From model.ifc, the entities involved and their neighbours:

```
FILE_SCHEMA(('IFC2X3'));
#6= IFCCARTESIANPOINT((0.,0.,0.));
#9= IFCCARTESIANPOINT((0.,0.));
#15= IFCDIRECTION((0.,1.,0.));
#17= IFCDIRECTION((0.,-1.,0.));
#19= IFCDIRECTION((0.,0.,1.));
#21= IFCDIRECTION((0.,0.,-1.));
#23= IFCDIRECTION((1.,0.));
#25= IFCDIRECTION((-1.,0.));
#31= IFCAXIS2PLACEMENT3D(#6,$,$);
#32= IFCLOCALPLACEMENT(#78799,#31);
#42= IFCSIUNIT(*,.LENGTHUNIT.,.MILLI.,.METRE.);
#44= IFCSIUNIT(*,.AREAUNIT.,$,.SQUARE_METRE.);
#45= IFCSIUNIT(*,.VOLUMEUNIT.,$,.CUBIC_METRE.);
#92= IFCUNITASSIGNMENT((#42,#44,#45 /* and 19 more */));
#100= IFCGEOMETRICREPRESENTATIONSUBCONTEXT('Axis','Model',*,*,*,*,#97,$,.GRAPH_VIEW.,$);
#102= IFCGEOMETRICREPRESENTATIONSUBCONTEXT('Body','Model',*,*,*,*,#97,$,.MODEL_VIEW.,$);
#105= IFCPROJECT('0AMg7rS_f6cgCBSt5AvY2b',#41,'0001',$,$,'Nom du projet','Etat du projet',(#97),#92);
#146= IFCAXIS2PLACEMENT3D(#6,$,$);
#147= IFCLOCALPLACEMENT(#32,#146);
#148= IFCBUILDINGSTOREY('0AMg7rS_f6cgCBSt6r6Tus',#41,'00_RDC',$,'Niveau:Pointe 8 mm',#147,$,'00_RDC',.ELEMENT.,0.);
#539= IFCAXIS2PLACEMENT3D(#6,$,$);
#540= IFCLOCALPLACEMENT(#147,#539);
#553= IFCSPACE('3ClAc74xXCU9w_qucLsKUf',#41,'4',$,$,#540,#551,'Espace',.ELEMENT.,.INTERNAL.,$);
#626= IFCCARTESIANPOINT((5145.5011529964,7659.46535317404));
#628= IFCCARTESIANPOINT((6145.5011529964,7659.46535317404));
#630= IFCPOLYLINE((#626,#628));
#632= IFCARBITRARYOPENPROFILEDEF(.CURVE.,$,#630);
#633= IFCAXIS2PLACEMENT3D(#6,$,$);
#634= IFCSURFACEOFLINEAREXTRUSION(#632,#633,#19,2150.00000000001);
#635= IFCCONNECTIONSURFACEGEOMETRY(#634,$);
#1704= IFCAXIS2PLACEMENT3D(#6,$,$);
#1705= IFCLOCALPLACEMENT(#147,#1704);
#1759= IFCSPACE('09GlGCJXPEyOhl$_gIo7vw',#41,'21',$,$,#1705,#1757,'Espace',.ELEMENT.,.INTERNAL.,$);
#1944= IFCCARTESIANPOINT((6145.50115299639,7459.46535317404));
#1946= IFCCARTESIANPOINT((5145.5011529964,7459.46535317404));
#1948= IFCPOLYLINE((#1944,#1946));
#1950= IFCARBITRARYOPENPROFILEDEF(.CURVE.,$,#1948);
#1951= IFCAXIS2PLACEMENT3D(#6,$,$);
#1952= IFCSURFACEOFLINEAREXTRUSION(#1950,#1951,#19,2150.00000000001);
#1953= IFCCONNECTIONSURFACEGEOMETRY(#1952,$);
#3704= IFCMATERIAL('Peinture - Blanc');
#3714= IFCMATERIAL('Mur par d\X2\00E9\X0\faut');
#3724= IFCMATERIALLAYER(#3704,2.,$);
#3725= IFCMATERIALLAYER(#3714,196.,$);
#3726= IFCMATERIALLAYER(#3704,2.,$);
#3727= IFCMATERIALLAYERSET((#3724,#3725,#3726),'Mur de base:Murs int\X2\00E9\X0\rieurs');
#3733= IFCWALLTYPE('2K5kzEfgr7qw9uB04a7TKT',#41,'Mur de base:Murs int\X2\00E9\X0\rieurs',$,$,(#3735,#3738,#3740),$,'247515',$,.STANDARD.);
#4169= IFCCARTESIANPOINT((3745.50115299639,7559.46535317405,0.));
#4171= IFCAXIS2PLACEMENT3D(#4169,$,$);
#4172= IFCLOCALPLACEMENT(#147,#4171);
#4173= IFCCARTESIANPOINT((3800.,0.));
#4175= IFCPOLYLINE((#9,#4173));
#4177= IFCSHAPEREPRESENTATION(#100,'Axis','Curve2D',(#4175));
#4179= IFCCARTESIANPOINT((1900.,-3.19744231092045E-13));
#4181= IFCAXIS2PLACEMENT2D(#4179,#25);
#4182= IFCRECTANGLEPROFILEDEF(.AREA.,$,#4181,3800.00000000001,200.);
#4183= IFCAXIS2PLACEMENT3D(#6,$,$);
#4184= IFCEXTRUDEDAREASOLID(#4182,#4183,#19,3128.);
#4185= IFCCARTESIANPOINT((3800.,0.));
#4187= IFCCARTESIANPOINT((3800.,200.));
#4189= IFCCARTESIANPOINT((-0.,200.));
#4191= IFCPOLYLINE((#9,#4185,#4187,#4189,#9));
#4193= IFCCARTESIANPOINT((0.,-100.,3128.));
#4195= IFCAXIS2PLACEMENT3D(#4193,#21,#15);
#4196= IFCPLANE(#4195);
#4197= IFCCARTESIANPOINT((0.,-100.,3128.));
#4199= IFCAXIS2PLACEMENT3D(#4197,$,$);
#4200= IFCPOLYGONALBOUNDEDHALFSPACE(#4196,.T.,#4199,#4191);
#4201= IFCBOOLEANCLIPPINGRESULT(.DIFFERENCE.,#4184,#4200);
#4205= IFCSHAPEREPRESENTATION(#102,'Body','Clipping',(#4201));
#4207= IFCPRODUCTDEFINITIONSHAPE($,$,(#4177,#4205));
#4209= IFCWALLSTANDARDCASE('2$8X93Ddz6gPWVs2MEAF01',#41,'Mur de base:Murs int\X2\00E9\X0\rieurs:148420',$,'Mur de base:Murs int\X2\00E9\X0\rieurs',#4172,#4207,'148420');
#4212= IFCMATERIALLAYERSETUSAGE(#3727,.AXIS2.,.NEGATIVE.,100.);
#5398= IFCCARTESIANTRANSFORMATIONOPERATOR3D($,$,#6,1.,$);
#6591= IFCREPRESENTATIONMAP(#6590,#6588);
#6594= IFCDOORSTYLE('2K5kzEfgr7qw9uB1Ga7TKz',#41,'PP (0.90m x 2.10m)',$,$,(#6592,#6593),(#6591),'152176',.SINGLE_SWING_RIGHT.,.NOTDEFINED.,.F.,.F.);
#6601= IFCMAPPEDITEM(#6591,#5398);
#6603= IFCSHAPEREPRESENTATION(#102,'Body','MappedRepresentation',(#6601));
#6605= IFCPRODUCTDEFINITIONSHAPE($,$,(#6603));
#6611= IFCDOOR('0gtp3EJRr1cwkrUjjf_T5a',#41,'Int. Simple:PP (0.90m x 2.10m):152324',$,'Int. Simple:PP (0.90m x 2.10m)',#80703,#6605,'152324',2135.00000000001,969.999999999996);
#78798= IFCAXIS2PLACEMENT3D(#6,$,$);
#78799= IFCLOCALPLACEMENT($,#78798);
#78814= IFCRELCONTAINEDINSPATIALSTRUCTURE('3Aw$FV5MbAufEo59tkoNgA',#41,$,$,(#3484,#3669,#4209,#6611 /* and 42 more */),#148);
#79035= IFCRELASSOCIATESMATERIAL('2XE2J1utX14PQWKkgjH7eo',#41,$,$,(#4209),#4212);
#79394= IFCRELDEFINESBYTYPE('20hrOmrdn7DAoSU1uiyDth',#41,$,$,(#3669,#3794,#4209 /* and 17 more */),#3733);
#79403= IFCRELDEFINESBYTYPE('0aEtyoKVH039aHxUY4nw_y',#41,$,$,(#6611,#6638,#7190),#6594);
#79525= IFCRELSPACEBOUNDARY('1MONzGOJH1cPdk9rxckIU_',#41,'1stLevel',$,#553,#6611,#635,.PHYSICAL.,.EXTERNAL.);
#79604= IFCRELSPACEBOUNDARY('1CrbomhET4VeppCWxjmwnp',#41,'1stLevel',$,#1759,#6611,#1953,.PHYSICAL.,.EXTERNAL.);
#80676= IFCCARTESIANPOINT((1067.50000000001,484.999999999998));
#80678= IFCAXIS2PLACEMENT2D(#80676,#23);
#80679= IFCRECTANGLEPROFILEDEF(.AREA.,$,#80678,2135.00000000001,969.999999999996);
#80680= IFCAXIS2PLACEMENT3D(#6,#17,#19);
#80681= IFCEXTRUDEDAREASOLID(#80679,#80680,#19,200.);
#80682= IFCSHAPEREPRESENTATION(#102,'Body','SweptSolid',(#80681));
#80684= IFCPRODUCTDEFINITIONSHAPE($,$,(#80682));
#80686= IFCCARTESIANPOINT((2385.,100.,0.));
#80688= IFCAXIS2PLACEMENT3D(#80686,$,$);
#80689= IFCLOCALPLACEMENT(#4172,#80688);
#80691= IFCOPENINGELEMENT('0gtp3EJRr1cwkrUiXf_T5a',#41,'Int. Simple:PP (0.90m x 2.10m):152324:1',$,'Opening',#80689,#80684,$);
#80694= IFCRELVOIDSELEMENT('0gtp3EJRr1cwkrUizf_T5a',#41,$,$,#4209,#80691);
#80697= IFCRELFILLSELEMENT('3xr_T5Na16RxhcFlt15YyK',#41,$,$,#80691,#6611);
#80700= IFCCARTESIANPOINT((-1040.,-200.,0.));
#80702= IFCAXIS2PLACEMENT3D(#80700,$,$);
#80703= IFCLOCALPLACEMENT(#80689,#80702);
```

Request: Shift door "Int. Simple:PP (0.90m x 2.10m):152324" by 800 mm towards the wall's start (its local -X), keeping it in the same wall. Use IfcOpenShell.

```python
import numpy as np
import ifcopenshell
import ifcopenshell.api.geometry
import ifcopenshell.util.placement

model = ifcopenshell.open("model.ifc")

door = model.by_id(6611)
opening = door.FillsVoids[0].RelatingOpeningElement
wall = opening.VoidsElements[0].RelatingBuildingElement

wall_matrix = ifcopenshell.util.placement.get_local_placement(wall.ObjectPlacement)
shift = wall_matrix[:3, 0] * -800.0
before = ifcopenshell.util.placement.get_local_placement(door.ObjectPlacement)[:3, 3].copy()

# The door is placed relative to its opening, so it follows when the opening moves.
matrix = ifcopenshell.util.placement.get_local_placement(opening.ObjectPlacement)
matrix[:3, 3] += shift
ifcopenshell.api.geometry.edit_object_placement(
    model, product=opening, matrix=matrix, is_si=False, should_transform_children=True
)

# Space boundary surfaces are stored in each space's coordinates; move them too.
for rel in door.ProvidesBoundaries:
    if not rel.ConnectionGeometry:
        continue
    surface = rel.ConnectionGeometry.SurfaceOnRelatingElement
    space_matrix = ifcopenshell.util.placement.get_local_placement(rel.RelatingSpace.ObjectPlacement)
    point = np.array(surface.Position.Location.Coordinates) + space_matrix[:3, :3].T @ shift
    surface.Position = model.createIfcAxis2Placement3D(
        model.createIfcCartesianPoint(point.tolist()), surface.Position.Axis, surface.Position.RefDirection
    )

after = ifcopenshell.util.placement.get_local_placement(door.ObjectPlacement)[:3, 3]
print("door moved by", (after - before).round(3) + 0.0)

model.write("model_edited.ifc")
```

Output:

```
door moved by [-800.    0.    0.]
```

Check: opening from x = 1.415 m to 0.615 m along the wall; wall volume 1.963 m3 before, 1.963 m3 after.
